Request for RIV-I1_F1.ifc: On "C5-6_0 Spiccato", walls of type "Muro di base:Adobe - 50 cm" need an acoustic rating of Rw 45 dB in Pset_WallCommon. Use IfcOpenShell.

First a look at what the model holds.

```python
import ifcopenshell
import ifcopenshell.util.element

model = ifcopenshell.open("RIV-I1_F1.ifc")
print(model.schema)
storey = next(s for s in model.by_type("IfcBuildingStorey") if s.Name == "C5-6_0 Spiccato")
walls = [e for e in ifcopenshell.util.element.get_decomposition(storey) if e.is_a("IfcWall")]
seen = {}
for e in walls:
    element_type = ifcopenshell.util.element.get_type(e)
    key = (element_type.Name if element_type != e and element_type else None, ifcopenshell.util.element.get_pset(e, "Pset_WallCommon", "AcousticRating"))
    seen[key] = seen.get(key, 0) + 1
for (name, value), count in sorted(seen.items(), key=str):
    print(count, "x", name, "|", value)
```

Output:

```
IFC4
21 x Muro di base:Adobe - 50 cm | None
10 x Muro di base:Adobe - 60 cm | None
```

```python
import ifcopenshell
import ifcopenshell.api.pset
import ifcopenshell.util.element

model = ifcopenshell.open("RIV-I1_F1.ifc")

storey = next(s for s in model.by_type("IfcBuildingStorey") if s.Name == "C5-6_0 Spiccato")
walls = [e for e in ifcopenshell.util.element.get_decomposition(storey) if e.is_a("IfcWall")]

count = 0
for e in walls:
    element_type = ifcopenshell.util.element.get_type(e)
    if element_type in (None, e) or element_type.Name != "Muro di base:Adobe - 50 cm":
        continue
    # add_pset returns the element's existing set when there is one.
    pset = ifcopenshell.api.pset.add_pset(model, product=e, name="Pset_WallCommon")
    ifcopenshell.api.pset.edit_pset(model, pset=pset, properties={"AcousticRating": "Rw 45 dB"})
    count += 1

print(count, "walls updated")

model.write("RIV-I1_F1_rev.ifc")
```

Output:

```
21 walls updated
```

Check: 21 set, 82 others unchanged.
